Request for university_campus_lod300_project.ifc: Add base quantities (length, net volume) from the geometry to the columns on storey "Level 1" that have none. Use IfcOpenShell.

First a look at what the model holds.

```python
import ifcopenshell
import ifcopenshell.util.element
import ifcopenshell.util.unit

model = ifcopenshell.open("university_campus_lod300_project.ifc")
print(model.schema)
for unit_type in ("LENGTHUNIT", "AREAUNIT", "VOLUMEUNIT"):
    print(unit_type, ifcopenshell.util.unit.calculate_unit_scale(model, unit_type))
storey = next(s for s in model.by_type("IfcBuildingStorey") if s.Name == "Level 1")
columns = [e for e in ifcopenshell.util.element.get_decomposition(storey) if e.is_a("IfcColumn")]
for e in sorted(columns, key=lambda e: e.id()):
    print(e.id(), e.is_a(), e.Name, list(ifcopenshell.util.element.get_psets(e, qtos_only=True)), sep=" | ")
```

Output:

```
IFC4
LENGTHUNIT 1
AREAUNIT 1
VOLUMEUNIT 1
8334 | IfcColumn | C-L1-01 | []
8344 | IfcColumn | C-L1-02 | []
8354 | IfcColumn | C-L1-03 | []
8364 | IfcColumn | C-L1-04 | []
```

```python
import ifcopenshell
import ifcopenshell.api.pset
import ifcopenshell.geom
import ifcopenshell.util.element
import ifcopenshell.util.shape
import ifcopenshell.util.unit

model = ifcopenshell.open("university_campus_lod300_project.ifc")
unit_scale = ifcopenshell.util.unit.calculate_unit_scale(model)
volume_scale = ifcopenshell.util.unit.calculate_unit_scale(model, "VOLUMEUNIT")
settings = ifcopenshell.geom.settings()

storey = next(s for s in model.by_type("IfcBuildingStorey") if s.Name == "Level 1")
columns = [e for e in ifcopenshell.util.element.get_decomposition(storey) if e.is_a("IfcColumn")]

for e in sorted(columns, key=lambda e: e.id()):
    if ifcopenshell.util.element.get_psets(e, qtos_only=True, should_inherit=False):
        continue
    # Geometry comes back in metres, in the element's own axes.
    shape = ifcopenshell.geom.create_shape(settings, e)
    values = {
        "Length": ifcopenshell.util.shape.get_z(shape.geometry) / unit_scale,
        "NetVolume": ifcopenshell.util.shape.get_volume(shape.geometry) / volume_scale,
    }
    qto = ifcopenshell.api.pset.add_qto(model, product=e, name="Qto_ColumnBaseQuantities")
    ifcopenshell.api.pset.edit_qto(model, qto=qto, properties=values)
    print(e.id(), {k: round(v, 3) for k, v in values.items()})

model.write("university_campus_lod300_project_edited.ifc")
```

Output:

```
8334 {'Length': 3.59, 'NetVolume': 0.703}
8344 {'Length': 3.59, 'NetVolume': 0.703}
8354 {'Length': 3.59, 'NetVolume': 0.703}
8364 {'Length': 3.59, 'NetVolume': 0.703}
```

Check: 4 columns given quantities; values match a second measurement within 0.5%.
